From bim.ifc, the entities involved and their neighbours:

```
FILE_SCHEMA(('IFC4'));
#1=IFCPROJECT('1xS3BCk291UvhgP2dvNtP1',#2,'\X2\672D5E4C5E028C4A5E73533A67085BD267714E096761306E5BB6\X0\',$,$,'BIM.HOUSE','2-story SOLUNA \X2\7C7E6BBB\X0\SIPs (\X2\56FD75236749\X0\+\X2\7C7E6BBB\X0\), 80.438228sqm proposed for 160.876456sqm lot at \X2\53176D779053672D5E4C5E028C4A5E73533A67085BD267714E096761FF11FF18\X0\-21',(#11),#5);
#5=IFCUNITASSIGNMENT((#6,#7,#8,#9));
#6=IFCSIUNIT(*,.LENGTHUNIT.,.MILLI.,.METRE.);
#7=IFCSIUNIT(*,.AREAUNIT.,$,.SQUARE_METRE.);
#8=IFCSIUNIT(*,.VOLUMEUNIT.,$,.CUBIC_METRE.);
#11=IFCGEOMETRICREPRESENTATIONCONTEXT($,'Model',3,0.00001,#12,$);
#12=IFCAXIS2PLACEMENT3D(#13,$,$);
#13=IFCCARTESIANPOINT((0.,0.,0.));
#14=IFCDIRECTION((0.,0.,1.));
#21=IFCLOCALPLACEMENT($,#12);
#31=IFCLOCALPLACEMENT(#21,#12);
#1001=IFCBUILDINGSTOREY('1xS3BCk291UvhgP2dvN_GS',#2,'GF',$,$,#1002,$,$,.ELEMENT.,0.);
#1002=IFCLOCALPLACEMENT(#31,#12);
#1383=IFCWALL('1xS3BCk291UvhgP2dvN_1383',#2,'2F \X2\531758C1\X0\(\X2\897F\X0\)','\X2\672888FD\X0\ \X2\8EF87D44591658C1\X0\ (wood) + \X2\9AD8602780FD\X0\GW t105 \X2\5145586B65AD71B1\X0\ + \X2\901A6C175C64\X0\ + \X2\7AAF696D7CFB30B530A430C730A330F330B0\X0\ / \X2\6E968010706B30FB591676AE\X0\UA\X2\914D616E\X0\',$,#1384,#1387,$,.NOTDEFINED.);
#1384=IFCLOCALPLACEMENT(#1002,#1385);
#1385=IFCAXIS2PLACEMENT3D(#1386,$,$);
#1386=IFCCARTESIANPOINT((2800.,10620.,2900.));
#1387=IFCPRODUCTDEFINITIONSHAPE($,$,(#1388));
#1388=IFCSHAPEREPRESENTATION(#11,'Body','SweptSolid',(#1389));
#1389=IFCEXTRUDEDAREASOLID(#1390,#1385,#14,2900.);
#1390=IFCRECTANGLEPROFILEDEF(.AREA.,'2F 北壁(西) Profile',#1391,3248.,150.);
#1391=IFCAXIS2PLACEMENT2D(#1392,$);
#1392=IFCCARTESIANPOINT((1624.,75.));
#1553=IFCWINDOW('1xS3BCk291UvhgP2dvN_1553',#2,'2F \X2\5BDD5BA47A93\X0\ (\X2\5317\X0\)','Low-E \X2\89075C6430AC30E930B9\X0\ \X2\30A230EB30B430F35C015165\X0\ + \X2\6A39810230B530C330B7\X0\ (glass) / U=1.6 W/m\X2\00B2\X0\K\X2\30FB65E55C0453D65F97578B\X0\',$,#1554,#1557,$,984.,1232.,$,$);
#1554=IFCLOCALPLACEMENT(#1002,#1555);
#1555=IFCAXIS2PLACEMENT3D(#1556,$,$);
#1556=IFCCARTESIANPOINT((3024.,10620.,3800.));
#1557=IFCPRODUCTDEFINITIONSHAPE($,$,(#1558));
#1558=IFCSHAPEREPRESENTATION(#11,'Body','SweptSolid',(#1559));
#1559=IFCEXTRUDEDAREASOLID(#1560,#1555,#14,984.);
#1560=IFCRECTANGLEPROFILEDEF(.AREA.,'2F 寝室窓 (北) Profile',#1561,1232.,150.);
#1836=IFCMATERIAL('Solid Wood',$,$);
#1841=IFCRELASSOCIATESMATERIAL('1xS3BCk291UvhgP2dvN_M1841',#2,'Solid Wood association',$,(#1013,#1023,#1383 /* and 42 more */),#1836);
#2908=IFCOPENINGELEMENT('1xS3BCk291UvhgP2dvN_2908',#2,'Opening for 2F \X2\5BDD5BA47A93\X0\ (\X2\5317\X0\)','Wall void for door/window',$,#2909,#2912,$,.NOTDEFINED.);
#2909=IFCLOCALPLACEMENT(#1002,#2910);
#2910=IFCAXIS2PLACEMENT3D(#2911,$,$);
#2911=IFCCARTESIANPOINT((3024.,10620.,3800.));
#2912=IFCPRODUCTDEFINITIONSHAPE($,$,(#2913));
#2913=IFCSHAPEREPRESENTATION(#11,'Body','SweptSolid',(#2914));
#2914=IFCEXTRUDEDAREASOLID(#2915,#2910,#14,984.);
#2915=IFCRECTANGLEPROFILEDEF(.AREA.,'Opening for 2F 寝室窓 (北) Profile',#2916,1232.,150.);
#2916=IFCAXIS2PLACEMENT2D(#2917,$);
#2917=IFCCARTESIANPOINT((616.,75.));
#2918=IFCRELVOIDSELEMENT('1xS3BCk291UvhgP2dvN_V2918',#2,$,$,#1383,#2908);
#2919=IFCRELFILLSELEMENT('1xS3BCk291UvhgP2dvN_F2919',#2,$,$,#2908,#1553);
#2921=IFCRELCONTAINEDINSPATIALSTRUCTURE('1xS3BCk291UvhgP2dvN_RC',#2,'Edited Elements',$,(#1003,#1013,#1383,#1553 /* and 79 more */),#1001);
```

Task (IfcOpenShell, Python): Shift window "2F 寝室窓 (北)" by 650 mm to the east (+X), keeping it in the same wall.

```python
import ifcopenshell
import ifcopenshell.api.geometry
import ifcopenshell.util.placement
import ifcopenshell.util.unit

model = ifcopenshell.open("bim.ifc")
unit_scale = ifcopenshell.util.unit.calculate_unit_scale(model)

window = model.by_guid("1xS3BCk291UvhgP2dvN_1553")
opening = window.FillsVoids[0].RelatingOpeningElement
wall = opening.VoidsElements[0].RelatingBuildingElement

wall_matrix = ifcopenshell.util.placement.get_local_placement(wall.ObjectPlacement)
shift = wall_matrix[:3, 0] * 0.65 / unit_scale
before = ifcopenshell.util.placement.get_local_placement(window.ObjectPlacement)[:3, 3].copy()

# The window is not placed relative to its opening, so move both.
for product in (opening, window):
    matrix = ifcopenshell.util.placement.get_local_placement(product.ObjectPlacement)
    matrix[:3, 3] += shift
    ifcopenshell.api.geometry.edit_object_placement(model, product=product, matrix=matrix, is_si=False)

after = ifcopenshell.util.placement.get_local_placement(window.ObjectPlacement)[:3, 3]
print("window moved by", (after - before).round(3) + 0.0)

model.write("bim_updated.ifc")
```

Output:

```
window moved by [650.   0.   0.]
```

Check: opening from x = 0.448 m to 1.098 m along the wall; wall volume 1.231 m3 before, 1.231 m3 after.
